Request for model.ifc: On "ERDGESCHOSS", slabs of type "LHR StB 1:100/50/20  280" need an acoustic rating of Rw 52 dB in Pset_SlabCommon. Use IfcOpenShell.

First a look at what the model holds.

```python
import ifcopenshell
import ifcopenshell.util.element

model = ifcopenshell.open("model.ifc")
print(model.schema)
storey = next(s for s in model.by_type("IfcBuildingStorey") if s.Name == "ERDGESCHOSS")
slabs = [e for e in ifcopenshell.util.element.get_decomposition(storey) if e.is_a("IfcSlab")]
seen = {}
for e in slabs:
    element_type = ifcopenshell.util.element.get_type(e)
    key = (element_type.Name if element_type != e and element_type else None, ifcopenshell.util.element.get_pset(e, "Pset_SlabCommon", "AcousticRating"))
    seen[key] = seen.get(key, 0) + 1
for (name, value), count in sorted(seen.items(), key=str):
    print(count, "x", name, "|", value)
```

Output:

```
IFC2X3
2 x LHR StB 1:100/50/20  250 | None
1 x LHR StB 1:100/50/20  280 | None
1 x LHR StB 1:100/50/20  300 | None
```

```python
import ifcopenshell
import ifcopenshell.api.pset
import ifcopenshell.util.element

model = ifcopenshell.open("model.ifc")

storey = next(s for s in model.by_type("IfcBuildingStorey") if s.Name == "ERDGESCHOSS")
slabs = [e for e in ifcopenshell.util.element.get_decomposition(storey) if e.is_a("IfcSlab")]

count = 0
for e in slabs:
    element_type = ifcopenshell.util.element.get_type(e)
    if element_type in (None, e) or element_type.Name != "LHR StB 1:100/50/20  280":
        continue
    # add_pset returns the element's existing set when there is one.
    pset = ifcopenshell.api.pset.add_pset(model, product=e, name="Pset_SlabCommon")
    ifcopenshell.api.pset.edit_pset(model, pset=pset, properties={"AcousticRating": "Rw 52 dB"})
    count += 1

print(count, "slabs updated")

model.write("model_edited.ifc")
```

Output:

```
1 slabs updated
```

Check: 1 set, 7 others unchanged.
